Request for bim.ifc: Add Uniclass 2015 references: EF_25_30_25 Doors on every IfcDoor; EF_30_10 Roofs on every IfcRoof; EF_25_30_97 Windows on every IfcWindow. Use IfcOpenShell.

First a look at what the model holds.

```python
import ifcopenshell

model = ifcopenshell.open("bim.ifc")
print(model.schema)
print("classifications:", [c.Name for c in model.by_type("IfcClassification")])
for ifc_class in ("IfcDoor", "IfcRoof", "IfcStair", "IfcWall", "IfcWindow"):
    print(ifc_class, len(model.by_type(ifc_class)))
```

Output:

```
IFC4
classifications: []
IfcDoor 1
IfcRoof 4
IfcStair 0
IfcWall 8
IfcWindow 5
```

```python
import ifcopenshell
import ifcopenshell.api.classification

model = ifcopenshell.open("bim.ifc")

system = ifcopenshell.api.classification.add_classification(model, classification="Uniclass 2015")

codes = {
    "IfcDoor": ("EF_25_30_25", "Doors"),
    "IfcRoof": ("EF_30_10", "Roofs"),
    "IfcWindow": ("EF_25_30_97", "Windows"),
}
for ifc_class, (code, name) in codes.items():
    products = model.by_type(ifc_class)
    ifcopenshell.api.classification.add_reference(
        model, products=products, classification=system, identification=code, name=name
    )
    print(code, len(products))

model.write("bim_v2.ifc")
```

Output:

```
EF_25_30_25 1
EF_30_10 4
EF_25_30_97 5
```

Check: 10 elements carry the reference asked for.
